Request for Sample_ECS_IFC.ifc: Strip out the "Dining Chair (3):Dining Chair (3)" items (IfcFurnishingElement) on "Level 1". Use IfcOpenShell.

First a look at what the model holds.

```python
import ifcopenshell
import ifcopenshell.util.element

model = ifcopenshell.open("Sample_ECS_IFC.ifc")
print(model.schema)
storey = next(s for s in model.by_type("IfcBuildingStorey") if s.Name == "Level 1")
furniture = [e for e in ifcopenshell.util.element.get_decomposition(storey) if e.is_a("IfcFurnishingElement")]
seen = {}
for e in furniture:
    element_type = ifcopenshell.util.element.get_type(e)
    name = element_type.Name if element_type not in (None, e) else None
    seen[name] = seen.get(name, 0) + 1
for name, count in sorted(seen.items(), key=str):
    print(count, "x", name)
```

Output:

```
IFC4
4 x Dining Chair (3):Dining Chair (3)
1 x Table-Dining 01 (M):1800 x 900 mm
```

```python
import ifcopenshell
import ifcopenshell.api.root
import ifcopenshell.util.element

model = ifcopenshell.open("Sample_ECS_IFC.ifc")

storey = next(s for s in model.by_type("IfcBuildingStorey") if s.Name == "Level 1")
furniture = [e for e in ifcopenshell.util.element.get_decomposition(storey) if e.is_a("IfcFurnishingElement")]
targets = [e for e in furniture if (t := ifcopenshell.util.element.get_type(e)) not in (None, e) and t.Name == "Dining Chair (3):Dining Chair (3)"]

for e in targets:
    ifcopenshell.api.root.remove_product(model, product=e)
print(len(targets), "removed")

model.write("Sample_ECS_IFC_updated.ifc")
```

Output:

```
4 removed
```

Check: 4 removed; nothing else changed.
